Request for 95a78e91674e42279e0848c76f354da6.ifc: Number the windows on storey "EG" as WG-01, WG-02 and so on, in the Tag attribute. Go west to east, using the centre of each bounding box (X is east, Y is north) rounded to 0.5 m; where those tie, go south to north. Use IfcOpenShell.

First a look at what the model holds.

```python
import ifcopenshell
import ifcopenshell.util.element
import ifcopenshell.util.placement

model = ifcopenshell.open("95a78e91674e42279e0848c76f354da6.ifc")
print(model.schema)
storey = next(s for s in model.by_type("IfcBuildingStorey") if s.Name == "EG")
windows = [e for e in ifcopenshell.util.element.get_decomposition(storey) if e.is_a("IfcWindow")]
for e in sorted(windows, key=lambda e: e.id()):
    origin = ifcopenshell.util.placement.get_local_placement(e.ObjectPlacement)[:3, 3]
    print(e.id(), e.Tag, e.Name, origin.round(2) + 0.0, sep=" | ")
```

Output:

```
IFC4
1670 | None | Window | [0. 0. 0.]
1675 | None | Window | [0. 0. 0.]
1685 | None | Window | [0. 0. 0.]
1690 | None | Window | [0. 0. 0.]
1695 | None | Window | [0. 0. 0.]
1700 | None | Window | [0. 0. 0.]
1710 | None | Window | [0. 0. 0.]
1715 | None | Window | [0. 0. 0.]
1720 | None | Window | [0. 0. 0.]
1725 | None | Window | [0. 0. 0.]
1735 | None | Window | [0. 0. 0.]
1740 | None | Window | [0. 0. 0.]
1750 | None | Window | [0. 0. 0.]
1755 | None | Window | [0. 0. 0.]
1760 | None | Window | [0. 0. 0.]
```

```python
import ifcopenshell
import ifcopenshell.geom
import ifcopenshell.util.element
import ifcopenshell.util.shape

model = ifcopenshell.open("95a78e91674e42279e0848c76f354da6.ifc")
settings = ifcopenshell.geom.settings()
settings.set("use-world-coords", True)


def centre(element):
    shape = ifcopenshell.geom.create_shape(settings, element)
    return ifcopenshell.util.shape.get_bbox_centroid(shape.geometry)


storey = next(s for s in model.by_type("IfcBuildingStorey") if s.Name == "EG")
windows = [e for e in ifcopenshell.util.element.get_decomposition(storey) if e.is_a("IfcWindow")]

# Insertion points can sit at a corner or the storey origin, so sort by the geometry (in metres).
centres = {e: centre(e) for e in windows}
windows.sort(key=lambda e: (round(centres[e][0] / 0.5), centres[e][1]))

for i, e in enumerate(windows, start=1):
    number = f"WG-{i:02d}"
    e.Tag = number
    print(e.id(), number)

model.write("95a78e91674e42279e0848c76f354da6_edited.ifc")
```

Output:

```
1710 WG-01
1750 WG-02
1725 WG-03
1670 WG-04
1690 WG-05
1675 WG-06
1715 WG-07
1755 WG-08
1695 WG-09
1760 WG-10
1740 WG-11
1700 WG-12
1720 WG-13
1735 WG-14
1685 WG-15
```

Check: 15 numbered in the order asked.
